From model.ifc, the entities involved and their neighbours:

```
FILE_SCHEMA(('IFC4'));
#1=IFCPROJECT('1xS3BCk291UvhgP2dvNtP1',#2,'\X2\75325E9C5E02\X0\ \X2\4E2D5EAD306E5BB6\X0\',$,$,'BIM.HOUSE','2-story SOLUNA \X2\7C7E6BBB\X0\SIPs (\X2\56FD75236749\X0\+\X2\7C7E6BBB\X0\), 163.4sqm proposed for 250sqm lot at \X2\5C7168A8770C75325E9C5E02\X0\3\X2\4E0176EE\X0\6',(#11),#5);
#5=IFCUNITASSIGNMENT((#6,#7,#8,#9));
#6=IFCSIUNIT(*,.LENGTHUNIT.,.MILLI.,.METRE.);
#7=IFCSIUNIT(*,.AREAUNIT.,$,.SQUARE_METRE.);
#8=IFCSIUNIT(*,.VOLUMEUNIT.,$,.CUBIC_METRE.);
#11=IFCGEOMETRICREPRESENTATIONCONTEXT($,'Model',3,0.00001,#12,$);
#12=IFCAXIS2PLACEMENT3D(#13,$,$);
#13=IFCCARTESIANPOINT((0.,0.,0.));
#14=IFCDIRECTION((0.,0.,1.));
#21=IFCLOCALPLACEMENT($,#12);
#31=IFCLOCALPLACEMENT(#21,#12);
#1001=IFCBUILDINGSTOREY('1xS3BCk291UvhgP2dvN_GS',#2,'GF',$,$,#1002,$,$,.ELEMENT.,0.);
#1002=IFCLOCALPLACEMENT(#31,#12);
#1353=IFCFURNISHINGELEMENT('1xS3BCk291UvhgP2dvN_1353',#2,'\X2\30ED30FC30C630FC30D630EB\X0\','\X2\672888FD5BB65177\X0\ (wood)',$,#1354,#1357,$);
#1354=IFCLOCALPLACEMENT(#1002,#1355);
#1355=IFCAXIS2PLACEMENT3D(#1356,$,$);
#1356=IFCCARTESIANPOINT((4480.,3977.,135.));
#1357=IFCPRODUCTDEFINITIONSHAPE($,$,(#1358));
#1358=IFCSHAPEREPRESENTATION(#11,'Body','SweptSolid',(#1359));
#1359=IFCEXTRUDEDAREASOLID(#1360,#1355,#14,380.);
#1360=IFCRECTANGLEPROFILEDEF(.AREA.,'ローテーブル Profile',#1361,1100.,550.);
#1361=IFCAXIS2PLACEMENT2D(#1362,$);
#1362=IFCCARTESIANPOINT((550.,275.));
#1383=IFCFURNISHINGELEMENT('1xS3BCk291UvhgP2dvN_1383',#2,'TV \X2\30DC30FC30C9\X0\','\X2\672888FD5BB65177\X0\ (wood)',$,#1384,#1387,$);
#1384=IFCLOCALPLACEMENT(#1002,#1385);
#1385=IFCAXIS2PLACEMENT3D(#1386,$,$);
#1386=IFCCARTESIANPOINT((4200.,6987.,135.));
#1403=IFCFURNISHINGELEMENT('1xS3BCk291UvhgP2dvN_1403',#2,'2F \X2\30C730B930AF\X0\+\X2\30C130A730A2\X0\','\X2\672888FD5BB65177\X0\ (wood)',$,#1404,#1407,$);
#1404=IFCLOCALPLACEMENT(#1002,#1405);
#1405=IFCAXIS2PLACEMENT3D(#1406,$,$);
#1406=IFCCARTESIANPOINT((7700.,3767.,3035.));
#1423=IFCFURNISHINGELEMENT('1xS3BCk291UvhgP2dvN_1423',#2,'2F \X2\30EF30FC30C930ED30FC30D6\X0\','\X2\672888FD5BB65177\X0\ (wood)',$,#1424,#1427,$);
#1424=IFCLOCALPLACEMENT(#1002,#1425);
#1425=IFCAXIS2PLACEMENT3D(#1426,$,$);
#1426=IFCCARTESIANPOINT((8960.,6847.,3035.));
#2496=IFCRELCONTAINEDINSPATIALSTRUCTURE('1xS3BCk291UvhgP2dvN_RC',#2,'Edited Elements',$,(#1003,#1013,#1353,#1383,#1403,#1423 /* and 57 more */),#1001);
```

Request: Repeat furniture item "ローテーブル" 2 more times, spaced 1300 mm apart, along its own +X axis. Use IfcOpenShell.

```python
import ifcopenshell
import ifcopenshell.api.geometry
import ifcopenshell.api.root
import ifcopenshell.util.element
import ifcopenshell.util.placement
import ifcopenshell.util.unit

model = ifcopenshell.open("model.ifc")
unit_scale = ifcopenshell.util.unit.calculate_unit_scale(model)


def reuse_history(source, copy):
    """copy_class also copies each property set's owner history, people and application; keep the originals."""
    for rel in copy.IsDefinedBy:
        if rel.is_a("IfcRelDefinesByProperties") and (history := rel.RelatingPropertyDefinition.OwnerHistory):
            rel.RelatingPropertyDefinition.OwnerHistory = source.OwnerHistory
            ifcopenshell.util.element.remove_deep2(model, history)


source = model.by_guid("1xS3BCk291UvhgP2dvN_1353")
base = ifcopenshell.util.placement.get_local_placement(source.ObjectPlacement)
step = base[:3, 0] * 1.3 / unit_scale

for i in range(1, 3):
    copy = ifcopenshell.api.root.copy_class(model, product=source)
    copy.Representation = ifcopenshell.util.element.copy_deep(
        model, source.Representation, exclude=["IfcGeometricRepresentationContext", "IfcRepresentationMap"]
    )
    reuse_history(source, copy)
    matrix = base.copy()
    matrix[:3, 3] += i * step
    print("added at", matrix[:3, 3].round(3) + 0.0)
    ifcopenshell.api.geometry.edit_object_placement(model, product=copy, matrix=matrix, is_si=False)

model.write("model_edited.ifc")
```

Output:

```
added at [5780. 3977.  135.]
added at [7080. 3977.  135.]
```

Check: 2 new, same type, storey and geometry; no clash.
